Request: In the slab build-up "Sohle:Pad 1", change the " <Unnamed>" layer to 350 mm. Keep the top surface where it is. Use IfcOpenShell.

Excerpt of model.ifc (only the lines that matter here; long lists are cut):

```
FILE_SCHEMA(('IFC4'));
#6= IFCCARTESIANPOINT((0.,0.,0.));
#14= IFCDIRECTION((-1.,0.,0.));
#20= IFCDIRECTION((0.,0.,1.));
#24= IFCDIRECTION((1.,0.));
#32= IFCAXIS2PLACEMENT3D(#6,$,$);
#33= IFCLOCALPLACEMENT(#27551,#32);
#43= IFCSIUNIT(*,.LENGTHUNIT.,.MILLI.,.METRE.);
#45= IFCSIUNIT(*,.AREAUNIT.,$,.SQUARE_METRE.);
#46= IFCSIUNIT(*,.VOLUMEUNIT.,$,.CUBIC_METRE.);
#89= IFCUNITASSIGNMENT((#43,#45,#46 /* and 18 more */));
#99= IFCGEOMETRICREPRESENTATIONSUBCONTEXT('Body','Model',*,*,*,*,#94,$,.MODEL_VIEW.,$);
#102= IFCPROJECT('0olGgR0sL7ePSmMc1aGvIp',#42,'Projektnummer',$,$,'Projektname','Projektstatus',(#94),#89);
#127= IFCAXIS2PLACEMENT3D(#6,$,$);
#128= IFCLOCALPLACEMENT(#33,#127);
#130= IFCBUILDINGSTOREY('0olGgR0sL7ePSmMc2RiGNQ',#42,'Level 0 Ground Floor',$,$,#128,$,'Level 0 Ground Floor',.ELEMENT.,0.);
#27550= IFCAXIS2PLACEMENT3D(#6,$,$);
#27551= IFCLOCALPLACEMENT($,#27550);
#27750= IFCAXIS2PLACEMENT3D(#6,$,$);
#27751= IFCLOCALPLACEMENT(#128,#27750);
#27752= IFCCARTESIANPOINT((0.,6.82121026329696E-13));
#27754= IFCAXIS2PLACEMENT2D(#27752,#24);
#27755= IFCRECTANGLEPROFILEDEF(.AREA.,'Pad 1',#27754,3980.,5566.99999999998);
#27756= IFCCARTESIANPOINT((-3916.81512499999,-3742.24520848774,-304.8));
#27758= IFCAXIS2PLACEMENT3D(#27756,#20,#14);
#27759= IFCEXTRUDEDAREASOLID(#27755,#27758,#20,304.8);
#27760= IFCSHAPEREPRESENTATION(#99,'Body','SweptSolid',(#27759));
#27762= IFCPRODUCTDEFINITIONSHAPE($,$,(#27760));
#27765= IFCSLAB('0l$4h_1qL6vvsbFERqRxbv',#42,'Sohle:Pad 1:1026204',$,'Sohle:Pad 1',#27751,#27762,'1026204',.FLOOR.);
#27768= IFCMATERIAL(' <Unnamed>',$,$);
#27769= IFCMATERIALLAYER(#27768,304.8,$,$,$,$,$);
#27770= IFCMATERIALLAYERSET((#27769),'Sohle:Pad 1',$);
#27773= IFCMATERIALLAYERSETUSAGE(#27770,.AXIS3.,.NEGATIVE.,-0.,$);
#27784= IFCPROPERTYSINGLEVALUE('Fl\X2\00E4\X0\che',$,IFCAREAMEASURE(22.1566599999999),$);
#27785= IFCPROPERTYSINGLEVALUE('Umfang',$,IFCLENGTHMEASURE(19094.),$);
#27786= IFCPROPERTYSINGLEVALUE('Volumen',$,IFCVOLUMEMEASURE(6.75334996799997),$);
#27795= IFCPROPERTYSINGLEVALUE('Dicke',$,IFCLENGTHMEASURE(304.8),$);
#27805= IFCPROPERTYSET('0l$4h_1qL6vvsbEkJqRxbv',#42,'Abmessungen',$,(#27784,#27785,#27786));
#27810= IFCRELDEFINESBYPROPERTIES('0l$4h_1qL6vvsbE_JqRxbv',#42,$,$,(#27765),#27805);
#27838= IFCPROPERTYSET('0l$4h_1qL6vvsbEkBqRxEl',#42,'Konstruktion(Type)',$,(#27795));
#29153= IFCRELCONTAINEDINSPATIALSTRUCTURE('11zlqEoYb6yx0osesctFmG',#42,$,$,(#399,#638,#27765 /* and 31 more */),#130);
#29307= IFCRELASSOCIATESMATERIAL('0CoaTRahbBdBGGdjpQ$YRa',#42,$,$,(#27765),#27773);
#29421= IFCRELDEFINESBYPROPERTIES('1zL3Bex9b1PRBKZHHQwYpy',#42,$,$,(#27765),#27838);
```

```python
import ifcopenshell
import ifcopenshell.api.pset
import ifcopenshell.util.element
import ifcopenshell.util.representation
import ifcopenshell.util.unit

model = ifcopenshell.open("model.ifc")
unit_scale = ifcopenshell.util.unit.calculate_unit_scale(model)

layer_set = model.by_id(27770)
layer = next(l for l in layer_set.MaterialLayers if l.Material and l.Material.Name == " <Unnamed>")
change = 0.35 / unit_scale - layer.LayerThickness
layer.LayerThickness += change

# Geometry does not follow the layer set by itself.
slabs = [e for e in ifcopenshell.util.element.get_elements_by_material(model, layer_set) if e.is_a("IfcSlab")]
for slab in sorted(slabs, key=lambda e: e.id()):
    body = ifcopenshell.util.representation.get_representation(slab, "Model", "Body")
    solid = body.Items[0]
    old_depth = solid.Depth
    solid.Depth += change
    # Extruded upwards: lower the start of the extrusion so the top stays.
    x, y, z = solid.Position.Location.Coordinates
    solid.Position.Location = model.createIfcCartesianPoint((x, y, z - change))
    pset = model.by_id(ifcopenshell.util.element.get_pset(slab, "Abmessungen", should_inherit=False)["id"])
    ifcopenshell.api.pset.edit_pset(model, pset=pset, properties={
        "Volumen": model.create_entity("IfcVolumeMeasure", ifcopenshell.util.element.get_pset(slab, "Abmessungen", "Volumen") * solid.Depth / old_depth),
    })
    pset = model.by_id(ifcopenshell.util.element.get_pset(slab, "Konstruktion(Type)", should_inherit=False)["id"])
    ifcopenshell.api.pset.edit_pset(model, pset=pset, properties={
        "Dicke": model.create_entity("IfcLengthMeasure", solid.Depth),
    })
    print(slab.id(), f"{old_depth:g} -> {solid.Depth:g}")

model.write("model_edited.ifc")
```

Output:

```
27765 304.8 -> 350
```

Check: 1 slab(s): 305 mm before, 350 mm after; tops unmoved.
